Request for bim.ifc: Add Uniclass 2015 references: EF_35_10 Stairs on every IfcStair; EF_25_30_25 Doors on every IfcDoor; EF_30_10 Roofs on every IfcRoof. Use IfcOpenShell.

First a look at what the model holds.

```python
import ifcopenshell

model = ifcopenshell.open("bim.ifc")
print(model.schema)
print("classifications:", [c.Name for c in model.by_type("IfcClassification")])
for ifc_class in ("IfcDoor", "IfcRoof", "IfcStair", "IfcWall", "IfcWindow"):
    print(ifc_class, len(model.by_type(ifc_class)))
```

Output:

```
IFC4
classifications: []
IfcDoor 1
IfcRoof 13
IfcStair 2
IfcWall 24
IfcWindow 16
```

```python
import ifcopenshell
import ifcopenshell.api.classification

model = ifcopenshell.open("bim.ifc")

system = ifcopenshell.api.classification.add_classification(model, classification="Uniclass 2015")

codes = {
    "IfcStair": ("EF_35_10", "Stairs"),
    "IfcDoor": ("EF_25_30_25", "Doors"),
    "IfcRoof": ("EF_30_10", "Roofs"),
}
for ifc_class, (code, name) in codes.items():
    products = model.by_type(ifc_class)
    ifcopenshell.api.classification.add_reference(
        model, products=products, classification=system, identification=code, name=name
    )
    print(code, len(products))

model.write("bim_edited.ifc")
```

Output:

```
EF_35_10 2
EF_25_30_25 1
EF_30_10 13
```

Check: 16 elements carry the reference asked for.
